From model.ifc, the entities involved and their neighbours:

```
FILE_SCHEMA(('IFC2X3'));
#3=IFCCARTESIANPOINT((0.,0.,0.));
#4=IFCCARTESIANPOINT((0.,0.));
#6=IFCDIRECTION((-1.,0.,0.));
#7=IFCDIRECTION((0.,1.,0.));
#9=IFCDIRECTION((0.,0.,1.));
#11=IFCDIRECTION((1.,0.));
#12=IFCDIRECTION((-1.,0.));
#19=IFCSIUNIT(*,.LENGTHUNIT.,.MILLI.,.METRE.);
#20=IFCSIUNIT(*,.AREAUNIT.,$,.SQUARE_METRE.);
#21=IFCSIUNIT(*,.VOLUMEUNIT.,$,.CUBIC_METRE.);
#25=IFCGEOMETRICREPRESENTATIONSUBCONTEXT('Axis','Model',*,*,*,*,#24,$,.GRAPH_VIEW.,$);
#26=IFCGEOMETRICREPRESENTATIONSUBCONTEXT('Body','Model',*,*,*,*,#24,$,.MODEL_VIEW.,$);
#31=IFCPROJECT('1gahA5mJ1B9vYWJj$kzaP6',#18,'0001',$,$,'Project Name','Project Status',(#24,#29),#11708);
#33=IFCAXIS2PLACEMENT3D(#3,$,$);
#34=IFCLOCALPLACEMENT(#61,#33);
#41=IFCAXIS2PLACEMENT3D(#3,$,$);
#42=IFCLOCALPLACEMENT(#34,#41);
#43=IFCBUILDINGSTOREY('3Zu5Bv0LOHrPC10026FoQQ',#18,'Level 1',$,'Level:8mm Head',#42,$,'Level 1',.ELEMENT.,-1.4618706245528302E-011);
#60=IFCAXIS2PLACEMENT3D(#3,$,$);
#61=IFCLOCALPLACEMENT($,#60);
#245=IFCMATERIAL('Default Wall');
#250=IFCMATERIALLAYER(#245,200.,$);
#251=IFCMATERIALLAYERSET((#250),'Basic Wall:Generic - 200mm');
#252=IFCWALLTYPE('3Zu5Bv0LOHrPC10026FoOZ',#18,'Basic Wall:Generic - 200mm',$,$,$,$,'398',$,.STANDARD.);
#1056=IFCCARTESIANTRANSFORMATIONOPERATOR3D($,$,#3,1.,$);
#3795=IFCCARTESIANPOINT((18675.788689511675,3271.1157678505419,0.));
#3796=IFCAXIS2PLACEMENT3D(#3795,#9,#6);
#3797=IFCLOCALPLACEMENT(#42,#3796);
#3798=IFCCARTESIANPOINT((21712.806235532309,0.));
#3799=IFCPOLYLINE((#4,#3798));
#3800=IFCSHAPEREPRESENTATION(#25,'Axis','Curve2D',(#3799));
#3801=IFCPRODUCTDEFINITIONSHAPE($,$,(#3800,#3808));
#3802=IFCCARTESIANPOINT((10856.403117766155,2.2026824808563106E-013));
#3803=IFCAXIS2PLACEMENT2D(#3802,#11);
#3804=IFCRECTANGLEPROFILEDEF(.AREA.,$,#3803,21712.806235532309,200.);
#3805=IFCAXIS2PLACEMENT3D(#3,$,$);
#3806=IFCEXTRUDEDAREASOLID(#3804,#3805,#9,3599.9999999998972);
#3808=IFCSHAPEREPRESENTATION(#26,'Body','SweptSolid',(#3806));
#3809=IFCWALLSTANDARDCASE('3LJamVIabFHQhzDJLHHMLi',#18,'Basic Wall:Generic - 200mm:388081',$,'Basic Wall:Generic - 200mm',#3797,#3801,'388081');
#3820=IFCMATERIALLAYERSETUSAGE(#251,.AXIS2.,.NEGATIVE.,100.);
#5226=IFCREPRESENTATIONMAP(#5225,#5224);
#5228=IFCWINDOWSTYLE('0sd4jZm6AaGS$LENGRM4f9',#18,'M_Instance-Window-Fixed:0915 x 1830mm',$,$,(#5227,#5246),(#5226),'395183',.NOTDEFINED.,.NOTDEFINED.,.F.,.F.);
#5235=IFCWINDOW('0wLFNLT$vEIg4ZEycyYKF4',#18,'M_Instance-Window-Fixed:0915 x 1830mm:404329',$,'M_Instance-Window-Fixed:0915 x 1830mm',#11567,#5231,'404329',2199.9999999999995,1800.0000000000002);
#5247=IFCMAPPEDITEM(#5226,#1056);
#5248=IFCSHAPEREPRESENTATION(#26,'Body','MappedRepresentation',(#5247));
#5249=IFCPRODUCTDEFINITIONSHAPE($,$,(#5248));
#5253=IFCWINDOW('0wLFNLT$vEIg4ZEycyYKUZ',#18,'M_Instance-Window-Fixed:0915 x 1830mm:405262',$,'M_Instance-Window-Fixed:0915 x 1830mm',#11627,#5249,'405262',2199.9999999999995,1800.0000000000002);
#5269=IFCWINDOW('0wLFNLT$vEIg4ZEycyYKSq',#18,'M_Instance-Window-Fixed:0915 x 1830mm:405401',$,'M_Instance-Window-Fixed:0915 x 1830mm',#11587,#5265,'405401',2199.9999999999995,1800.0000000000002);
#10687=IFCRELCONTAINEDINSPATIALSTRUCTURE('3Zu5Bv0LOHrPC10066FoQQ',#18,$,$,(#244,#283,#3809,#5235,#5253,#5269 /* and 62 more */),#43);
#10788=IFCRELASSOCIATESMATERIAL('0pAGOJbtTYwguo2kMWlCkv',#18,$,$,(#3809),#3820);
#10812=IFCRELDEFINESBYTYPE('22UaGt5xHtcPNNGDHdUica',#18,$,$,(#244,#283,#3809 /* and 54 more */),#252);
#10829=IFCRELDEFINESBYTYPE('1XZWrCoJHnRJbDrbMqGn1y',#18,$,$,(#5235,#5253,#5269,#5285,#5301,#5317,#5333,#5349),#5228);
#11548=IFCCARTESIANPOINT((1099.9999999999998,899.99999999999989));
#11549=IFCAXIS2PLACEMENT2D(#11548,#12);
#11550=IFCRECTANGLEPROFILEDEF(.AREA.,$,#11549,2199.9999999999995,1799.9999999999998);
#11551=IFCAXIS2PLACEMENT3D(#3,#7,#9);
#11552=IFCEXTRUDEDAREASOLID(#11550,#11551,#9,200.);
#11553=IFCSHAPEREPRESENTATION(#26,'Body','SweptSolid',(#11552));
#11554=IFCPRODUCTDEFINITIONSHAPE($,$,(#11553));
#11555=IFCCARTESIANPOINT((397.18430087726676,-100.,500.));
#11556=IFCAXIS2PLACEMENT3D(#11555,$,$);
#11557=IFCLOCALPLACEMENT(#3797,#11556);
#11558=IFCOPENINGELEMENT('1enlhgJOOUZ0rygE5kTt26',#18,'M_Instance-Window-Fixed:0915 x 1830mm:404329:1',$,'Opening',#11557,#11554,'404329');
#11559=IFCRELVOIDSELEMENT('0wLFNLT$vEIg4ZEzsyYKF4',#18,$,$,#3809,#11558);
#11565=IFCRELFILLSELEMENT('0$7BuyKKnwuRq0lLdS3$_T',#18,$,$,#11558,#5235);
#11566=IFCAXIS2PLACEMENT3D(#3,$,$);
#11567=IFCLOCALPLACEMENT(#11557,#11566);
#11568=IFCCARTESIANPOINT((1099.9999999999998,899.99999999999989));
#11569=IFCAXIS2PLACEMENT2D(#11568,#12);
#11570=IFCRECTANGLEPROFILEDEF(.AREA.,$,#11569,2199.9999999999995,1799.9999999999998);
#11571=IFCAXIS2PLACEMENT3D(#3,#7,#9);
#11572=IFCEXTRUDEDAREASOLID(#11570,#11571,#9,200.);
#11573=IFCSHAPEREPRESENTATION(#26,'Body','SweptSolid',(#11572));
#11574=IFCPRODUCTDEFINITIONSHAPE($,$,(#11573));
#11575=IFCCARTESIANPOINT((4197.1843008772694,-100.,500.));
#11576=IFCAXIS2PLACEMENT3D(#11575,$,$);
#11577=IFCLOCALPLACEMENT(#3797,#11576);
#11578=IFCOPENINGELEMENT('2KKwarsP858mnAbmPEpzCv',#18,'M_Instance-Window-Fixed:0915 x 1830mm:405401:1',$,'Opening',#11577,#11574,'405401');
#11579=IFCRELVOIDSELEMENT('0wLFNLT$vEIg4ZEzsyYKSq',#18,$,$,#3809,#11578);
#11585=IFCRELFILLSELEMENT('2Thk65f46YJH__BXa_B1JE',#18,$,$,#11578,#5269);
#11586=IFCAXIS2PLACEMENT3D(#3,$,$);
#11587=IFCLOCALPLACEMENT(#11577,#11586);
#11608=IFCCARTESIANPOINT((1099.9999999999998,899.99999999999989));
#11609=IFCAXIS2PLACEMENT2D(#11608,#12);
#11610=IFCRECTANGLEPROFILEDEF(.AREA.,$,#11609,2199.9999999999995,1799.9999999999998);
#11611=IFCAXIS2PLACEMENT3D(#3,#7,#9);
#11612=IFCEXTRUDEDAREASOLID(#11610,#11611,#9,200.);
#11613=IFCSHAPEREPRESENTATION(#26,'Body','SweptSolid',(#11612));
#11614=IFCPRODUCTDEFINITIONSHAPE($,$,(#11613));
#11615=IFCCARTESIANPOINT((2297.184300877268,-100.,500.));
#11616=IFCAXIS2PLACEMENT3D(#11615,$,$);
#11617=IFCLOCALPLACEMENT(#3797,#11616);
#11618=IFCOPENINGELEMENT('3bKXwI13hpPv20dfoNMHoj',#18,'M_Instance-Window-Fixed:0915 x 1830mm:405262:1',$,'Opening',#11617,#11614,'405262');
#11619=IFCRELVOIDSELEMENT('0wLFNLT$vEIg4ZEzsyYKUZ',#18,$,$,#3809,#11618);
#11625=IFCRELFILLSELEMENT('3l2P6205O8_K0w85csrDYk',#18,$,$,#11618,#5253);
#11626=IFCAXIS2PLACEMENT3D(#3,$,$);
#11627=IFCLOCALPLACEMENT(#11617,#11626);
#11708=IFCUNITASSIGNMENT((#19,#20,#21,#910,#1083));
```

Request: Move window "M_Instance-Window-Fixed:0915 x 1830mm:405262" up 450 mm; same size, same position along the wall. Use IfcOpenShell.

```python
import numpy as np
import ifcopenshell
import ifcopenshell.api.geometry
import ifcopenshell.util.placement
import ifcopenshell.util.unit

model = ifcopenshell.open("model.ifc")
unit_scale = ifcopenshell.util.unit.calculate_unit_scale(model)

window = model.by_guid("0wLFNLT$vEIg4ZEycyYKUZ")
opening = window.FillsVoids[0].RelatingOpeningElement
dz = 0.45 / unit_scale

shift = np.array([0.0, 0.0, dz])
# The window is placed relative to its opening, so it follows when the opening moves.
matrix = ifcopenshell.util.placement.get_local_placement(opening.ObjectPlacement)
matrix[:3, 3] += shift
ifcopenshell.api.geometry.edit_object_placement(
    model, product=opening, matrix=matrix, is_si=False, should_transform_children=True
)

print(f"moved by {dz * unit_scale:+.3f} m")

model.write("model_updated.ifc")
```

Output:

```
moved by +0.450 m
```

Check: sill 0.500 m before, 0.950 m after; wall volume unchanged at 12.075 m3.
